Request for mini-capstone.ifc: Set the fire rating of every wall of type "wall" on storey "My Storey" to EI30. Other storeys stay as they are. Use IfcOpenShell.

First a look at what the model holds.

```python
import ifcopenshell
import ifcopenshell.util.element

model = ifcopenshell.open("mini-capstone.ifc")
print(model.schema)
storey = next(s for s in model.by_type("IfcBuildingStorey") if s.Name == "My Storey")
walls = [e for e in ifcopenshell.util.element.get_decomposition(storey) if e.is_a("IfcWall")]
seen = {}
for e in walls:
    element_type = ifcopenshell.util.element.get_type(e)
    key = (element_type.Name if element_type != e and element_type else None, ifcopenshell.util.element.get_pset(e, "Pset_WallCommon", "FireRating"))
    seen[key] = seen.get(key, 0) + 1
for (name, value), count in sorted(seen.items(), key=str):
    print(count, "x", name, "|", value)
```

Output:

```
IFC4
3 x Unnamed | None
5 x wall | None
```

```python
import ifcopenshell
import ifcopenshell.api.pset
import ifcopenshell.util.element

model = ifcopenshell.open("mini-capstone.ifc")

storey = next(s for s in model.by_type("IfcBuildingStorey") if s.Name == "My Storey")
walls = [e for e in ifcopenshell.util.element.get_decomposition(storey) if e.is_a("IfcWall")]

count = 0
for e in walls:
    element_type = ifcopenshell.util.element.get_type(e)
    if element_type in (None, e) or element_type.Name != "wall":
        continue
    # add_pset returns the element's existing set when there is one.
    pset = ifcopenshell.api.pset.add_pset(model, product=e, name="Pset_WallCommon")
    ifcopenshell.api.pset.edit_pset(model, pset=pset, properties={"FireRating": "EI30"})
    count += 1

print(count, "walls updated")

model.write("mini-capstone_v2.ifc")
```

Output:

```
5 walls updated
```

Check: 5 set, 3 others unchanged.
